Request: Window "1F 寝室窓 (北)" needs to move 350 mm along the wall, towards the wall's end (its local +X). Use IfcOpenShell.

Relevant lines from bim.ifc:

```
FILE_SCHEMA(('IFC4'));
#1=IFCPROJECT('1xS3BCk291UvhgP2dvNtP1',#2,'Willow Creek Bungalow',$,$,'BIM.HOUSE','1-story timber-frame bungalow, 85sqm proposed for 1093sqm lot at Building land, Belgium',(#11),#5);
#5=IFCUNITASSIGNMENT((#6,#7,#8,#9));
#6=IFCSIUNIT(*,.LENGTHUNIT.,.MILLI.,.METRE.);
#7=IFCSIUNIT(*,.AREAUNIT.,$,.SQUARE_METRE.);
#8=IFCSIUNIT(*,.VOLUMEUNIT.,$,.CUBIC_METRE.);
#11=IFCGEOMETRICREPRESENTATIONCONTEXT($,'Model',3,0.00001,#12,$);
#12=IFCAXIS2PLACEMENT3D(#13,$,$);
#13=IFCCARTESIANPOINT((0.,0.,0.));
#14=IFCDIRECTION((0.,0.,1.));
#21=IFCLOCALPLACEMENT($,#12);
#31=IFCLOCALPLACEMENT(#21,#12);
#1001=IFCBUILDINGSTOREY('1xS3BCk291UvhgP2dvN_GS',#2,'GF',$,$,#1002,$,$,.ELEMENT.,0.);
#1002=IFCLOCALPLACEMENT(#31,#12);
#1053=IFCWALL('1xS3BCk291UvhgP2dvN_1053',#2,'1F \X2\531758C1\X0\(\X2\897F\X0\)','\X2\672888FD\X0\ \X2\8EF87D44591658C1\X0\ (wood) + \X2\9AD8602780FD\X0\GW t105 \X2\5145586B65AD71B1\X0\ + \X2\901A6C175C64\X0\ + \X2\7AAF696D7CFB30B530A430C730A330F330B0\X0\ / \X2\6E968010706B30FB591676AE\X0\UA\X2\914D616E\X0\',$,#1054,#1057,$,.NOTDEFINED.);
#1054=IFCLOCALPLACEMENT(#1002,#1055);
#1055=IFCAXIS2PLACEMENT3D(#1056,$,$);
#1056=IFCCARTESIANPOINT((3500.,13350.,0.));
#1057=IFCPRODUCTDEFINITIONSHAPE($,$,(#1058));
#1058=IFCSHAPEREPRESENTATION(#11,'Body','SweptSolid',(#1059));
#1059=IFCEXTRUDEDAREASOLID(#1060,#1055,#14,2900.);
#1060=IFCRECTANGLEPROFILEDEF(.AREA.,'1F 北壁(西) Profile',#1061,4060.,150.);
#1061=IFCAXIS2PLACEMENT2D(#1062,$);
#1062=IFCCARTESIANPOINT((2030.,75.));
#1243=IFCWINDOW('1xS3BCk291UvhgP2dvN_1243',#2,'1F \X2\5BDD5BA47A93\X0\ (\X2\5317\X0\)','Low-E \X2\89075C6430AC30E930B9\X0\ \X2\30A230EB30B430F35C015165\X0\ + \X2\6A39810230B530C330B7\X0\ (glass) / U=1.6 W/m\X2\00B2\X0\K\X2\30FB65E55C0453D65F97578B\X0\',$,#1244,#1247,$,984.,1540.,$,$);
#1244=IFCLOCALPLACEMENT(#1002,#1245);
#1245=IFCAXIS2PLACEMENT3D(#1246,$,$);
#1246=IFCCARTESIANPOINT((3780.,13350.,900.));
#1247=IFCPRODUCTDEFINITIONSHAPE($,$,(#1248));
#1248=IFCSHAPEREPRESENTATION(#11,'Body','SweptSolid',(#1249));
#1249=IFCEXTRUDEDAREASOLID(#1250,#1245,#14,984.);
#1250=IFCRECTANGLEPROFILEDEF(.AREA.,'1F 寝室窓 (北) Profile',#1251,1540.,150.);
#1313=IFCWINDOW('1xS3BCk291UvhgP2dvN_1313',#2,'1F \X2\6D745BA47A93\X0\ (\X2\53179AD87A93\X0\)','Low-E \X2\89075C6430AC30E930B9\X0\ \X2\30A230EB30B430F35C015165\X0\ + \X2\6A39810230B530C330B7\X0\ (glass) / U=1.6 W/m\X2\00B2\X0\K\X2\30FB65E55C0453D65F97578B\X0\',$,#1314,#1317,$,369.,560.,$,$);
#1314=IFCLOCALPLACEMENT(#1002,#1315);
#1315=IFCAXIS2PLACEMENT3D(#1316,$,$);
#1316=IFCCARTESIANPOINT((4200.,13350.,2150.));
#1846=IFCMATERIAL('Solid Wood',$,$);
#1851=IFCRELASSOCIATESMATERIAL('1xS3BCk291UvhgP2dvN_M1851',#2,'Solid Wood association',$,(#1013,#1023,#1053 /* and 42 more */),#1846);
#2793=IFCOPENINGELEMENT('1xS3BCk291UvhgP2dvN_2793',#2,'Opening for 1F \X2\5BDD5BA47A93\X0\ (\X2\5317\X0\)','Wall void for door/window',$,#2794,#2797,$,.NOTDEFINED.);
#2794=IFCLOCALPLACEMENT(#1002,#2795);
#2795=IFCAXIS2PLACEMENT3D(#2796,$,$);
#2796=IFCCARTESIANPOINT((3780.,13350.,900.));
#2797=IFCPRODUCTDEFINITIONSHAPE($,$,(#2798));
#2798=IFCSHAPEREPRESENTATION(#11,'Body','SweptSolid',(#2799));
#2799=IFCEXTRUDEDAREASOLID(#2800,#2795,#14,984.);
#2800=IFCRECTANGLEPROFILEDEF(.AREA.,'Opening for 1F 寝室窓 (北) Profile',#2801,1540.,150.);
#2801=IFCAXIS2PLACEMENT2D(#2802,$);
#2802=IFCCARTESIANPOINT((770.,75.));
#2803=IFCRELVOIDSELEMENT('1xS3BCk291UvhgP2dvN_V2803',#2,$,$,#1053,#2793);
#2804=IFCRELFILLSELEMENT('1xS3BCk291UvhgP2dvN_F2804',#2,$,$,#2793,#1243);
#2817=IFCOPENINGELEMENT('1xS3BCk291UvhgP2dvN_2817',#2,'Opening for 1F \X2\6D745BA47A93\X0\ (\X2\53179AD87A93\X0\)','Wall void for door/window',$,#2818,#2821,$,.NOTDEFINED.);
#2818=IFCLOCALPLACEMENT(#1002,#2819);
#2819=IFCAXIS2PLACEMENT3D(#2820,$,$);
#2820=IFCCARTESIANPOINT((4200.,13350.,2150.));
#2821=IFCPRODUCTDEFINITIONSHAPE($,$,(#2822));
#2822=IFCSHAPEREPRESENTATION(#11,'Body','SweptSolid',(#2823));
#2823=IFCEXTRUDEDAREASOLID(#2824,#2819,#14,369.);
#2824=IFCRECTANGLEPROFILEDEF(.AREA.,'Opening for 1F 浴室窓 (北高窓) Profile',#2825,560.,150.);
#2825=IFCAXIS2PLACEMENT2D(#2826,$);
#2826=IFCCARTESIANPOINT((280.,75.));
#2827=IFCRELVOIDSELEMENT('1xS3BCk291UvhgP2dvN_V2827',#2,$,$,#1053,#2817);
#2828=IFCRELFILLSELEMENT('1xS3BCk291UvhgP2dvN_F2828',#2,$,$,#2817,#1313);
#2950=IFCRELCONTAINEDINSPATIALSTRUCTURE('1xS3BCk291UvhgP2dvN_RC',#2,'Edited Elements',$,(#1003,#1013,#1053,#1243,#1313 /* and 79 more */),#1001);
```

```python
import ifcopenshell
import ifcopenshell.api.geometry
import ifcopenshell.util.placement

model = ifcopenshell.open("bim.ifc")

window = model.by_guid("1xS3BCk291UvhgP2dvN_1243")
opening = window.FillsVoids[0].RelatingOpeningElement
wall = opening.VoidsElements[0].RelatingBuildingElement

wall_matrix = ifcopenshell.util.placement.get_local_placement(wall.ObjectPlacement)
shift = wall_matrix[:3, 0] * 350.0
before = ifcopenshell.util.placement.get_local_placement(window.ObjectPlacement)[:3, 3].copy()

# The window is not placed relative to its opening, so move both.
for product in (opening, window):
    matrix = ifcopenshell.util.placement.get_local_placement(product.ObjectPlacement)
    matrix[:3, 3] += shift
    ifcopenshell.api.geometry.edit_object_placement(model, product=product, matrix=matrix, is_si=False)

after = ifcopenshell.util.placement.get_local_placement(window.ObjectPlacement)[:3, 3]
print("window moved by", (after - before).round(3) + 0.0)

model.write("bim_rev.ifc")
```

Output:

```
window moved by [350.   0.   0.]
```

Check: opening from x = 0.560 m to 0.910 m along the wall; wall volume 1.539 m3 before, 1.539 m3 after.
